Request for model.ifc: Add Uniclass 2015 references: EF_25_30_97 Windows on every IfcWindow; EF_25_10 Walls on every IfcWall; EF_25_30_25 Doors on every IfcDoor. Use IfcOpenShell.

First a look at what the model holds.

```python
import ifcopenshell

model = ifcopenshell.open("model.ifc")
print(model.schema)
print("classifications:", [c.Name for c in model.by_type("IfcClassification")])
for ifc_class in ("IfcDoor", "IfcRoof", "IfcStair", "IfcWall", "IfcWindow"):
    print(ifc_class, len(model.by_type(ifc_class)))
```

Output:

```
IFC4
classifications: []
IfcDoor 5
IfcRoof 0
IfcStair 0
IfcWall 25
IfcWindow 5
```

```python
import ifcopenshell
import ifcopenshell.api.classification

model = ifcopenshell.open("model.ifc")

system = ifcopenshell.api.classification.add_classification(model, classification="Uniclass 2015")

codes = {
    "IfcWindow": ("EF_25_30_97", "Windows"),
    "IfcWall": ("EF_25_10", "Walls"),
    "IfcDoor": ("EF_25_30_25", "Doors"),
}
for ifc_class, (code, name) in codes.items():
    products = model.by_type(ifc_class)
    ifcopenshell.api.classification.add_reference(
        model, products=products, classification=system, identification=code, name=name
    )
    print(code, len(products))

model.write("model-out.ifc")
```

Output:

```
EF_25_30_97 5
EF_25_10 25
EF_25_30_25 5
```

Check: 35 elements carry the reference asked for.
